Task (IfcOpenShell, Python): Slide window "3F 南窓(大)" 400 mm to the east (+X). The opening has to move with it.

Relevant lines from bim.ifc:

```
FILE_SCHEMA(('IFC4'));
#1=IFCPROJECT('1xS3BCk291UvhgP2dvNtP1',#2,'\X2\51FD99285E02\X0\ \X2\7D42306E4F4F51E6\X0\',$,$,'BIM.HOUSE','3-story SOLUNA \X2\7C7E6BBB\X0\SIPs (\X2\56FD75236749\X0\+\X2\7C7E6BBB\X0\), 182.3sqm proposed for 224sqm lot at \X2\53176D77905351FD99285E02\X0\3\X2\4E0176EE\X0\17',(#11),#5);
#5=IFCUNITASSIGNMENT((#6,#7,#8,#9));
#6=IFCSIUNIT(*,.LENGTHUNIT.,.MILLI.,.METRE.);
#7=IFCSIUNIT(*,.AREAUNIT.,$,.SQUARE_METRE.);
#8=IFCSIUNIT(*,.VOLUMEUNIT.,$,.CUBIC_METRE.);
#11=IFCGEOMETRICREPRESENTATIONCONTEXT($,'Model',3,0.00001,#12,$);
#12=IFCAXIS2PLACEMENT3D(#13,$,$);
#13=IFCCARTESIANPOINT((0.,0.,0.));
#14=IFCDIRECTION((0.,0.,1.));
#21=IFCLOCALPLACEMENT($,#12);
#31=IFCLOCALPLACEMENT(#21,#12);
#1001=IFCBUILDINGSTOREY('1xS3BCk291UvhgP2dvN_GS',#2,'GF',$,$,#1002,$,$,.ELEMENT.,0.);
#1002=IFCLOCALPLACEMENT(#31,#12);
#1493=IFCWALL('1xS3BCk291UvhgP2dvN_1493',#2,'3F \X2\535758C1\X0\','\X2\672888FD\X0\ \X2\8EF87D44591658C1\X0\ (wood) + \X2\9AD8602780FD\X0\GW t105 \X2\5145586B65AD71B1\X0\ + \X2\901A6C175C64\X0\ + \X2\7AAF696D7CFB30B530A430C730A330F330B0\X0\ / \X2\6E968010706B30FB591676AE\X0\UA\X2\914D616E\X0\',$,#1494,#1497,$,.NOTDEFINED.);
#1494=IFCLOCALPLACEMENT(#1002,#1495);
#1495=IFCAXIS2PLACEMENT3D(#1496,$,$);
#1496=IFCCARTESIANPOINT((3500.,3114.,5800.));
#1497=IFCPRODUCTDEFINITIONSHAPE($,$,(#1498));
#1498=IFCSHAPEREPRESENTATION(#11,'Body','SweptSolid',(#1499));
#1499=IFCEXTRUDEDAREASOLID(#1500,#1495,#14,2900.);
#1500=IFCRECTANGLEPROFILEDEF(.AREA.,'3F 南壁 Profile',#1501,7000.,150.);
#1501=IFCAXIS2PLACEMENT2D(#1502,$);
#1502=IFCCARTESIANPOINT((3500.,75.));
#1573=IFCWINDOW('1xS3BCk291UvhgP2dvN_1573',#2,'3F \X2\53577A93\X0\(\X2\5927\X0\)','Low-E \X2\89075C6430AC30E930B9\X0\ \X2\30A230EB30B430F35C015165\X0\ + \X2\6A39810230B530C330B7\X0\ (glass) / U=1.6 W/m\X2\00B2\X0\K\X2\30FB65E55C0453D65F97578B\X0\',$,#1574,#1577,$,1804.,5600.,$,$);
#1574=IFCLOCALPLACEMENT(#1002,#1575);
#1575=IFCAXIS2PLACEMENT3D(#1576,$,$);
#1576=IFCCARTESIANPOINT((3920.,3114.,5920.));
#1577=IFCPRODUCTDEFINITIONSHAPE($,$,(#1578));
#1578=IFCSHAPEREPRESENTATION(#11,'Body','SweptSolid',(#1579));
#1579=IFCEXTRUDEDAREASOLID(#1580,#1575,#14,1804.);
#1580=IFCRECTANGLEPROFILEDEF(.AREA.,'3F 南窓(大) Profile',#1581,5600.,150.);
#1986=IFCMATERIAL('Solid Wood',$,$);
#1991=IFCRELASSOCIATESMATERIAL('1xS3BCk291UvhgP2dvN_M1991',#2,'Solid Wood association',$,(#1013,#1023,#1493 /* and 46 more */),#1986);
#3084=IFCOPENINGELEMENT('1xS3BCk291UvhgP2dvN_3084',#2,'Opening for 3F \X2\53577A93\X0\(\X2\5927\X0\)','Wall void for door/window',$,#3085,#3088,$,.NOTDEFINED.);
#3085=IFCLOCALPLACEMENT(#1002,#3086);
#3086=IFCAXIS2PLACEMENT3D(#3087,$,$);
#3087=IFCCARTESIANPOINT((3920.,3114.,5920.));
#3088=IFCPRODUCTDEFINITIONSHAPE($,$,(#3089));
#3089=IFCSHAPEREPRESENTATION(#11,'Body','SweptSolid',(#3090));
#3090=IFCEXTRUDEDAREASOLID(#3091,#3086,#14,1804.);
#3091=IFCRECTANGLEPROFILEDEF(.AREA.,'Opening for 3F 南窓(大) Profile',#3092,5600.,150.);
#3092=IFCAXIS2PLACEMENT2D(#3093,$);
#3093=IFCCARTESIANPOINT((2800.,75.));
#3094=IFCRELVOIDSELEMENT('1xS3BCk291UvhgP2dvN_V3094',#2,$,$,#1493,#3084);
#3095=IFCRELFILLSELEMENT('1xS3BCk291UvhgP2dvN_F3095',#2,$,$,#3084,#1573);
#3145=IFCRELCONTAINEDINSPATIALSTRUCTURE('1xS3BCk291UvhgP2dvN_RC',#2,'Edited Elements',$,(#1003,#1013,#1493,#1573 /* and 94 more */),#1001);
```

```python
import ifcopenshell
import ifcopenshell.api.geometry
import ifcopenshell.util.placement

model = ifcopenshell.open("bim.ifc")

window = model.by_guid("1xS3BCk291UvhgP2dvN_1573")
opening = window.FillsVoids[0].RelatingOpeningElement
wall = opening.VoidsElements[0].RelatingBuildingElement

wall_matrix = ifcopenshell.util.placement.get_local_placement(wall.ObjectPlacement)
shift = wall_matrix[:3, 0] * 400.0
before = ifcopenshell.util.placement.get_local_placement(window.ObjectPlacement)[:3, 3].copy()

# The window is not placed relative to its opening, so move both.
for product in (opening, window):
    matrix = ifcopenshell.util.placement.get_local_placement(product.ObjectPlacement)
    matrix[:3, 3] += shift
    ifcopenshell.api.geometry.edit_object_placement(model, product=product, matrix=matrix, is_si=False)

after = ifcopenshell.util.placement.get_local_placement(window.ObjectPlacement)[:3, 3]
print("window moved by", (after - before).round(3) + 0.0)

model.write("bim_updated.ifc")
```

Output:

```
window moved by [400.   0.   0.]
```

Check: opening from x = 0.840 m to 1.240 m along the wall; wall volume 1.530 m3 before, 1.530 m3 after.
